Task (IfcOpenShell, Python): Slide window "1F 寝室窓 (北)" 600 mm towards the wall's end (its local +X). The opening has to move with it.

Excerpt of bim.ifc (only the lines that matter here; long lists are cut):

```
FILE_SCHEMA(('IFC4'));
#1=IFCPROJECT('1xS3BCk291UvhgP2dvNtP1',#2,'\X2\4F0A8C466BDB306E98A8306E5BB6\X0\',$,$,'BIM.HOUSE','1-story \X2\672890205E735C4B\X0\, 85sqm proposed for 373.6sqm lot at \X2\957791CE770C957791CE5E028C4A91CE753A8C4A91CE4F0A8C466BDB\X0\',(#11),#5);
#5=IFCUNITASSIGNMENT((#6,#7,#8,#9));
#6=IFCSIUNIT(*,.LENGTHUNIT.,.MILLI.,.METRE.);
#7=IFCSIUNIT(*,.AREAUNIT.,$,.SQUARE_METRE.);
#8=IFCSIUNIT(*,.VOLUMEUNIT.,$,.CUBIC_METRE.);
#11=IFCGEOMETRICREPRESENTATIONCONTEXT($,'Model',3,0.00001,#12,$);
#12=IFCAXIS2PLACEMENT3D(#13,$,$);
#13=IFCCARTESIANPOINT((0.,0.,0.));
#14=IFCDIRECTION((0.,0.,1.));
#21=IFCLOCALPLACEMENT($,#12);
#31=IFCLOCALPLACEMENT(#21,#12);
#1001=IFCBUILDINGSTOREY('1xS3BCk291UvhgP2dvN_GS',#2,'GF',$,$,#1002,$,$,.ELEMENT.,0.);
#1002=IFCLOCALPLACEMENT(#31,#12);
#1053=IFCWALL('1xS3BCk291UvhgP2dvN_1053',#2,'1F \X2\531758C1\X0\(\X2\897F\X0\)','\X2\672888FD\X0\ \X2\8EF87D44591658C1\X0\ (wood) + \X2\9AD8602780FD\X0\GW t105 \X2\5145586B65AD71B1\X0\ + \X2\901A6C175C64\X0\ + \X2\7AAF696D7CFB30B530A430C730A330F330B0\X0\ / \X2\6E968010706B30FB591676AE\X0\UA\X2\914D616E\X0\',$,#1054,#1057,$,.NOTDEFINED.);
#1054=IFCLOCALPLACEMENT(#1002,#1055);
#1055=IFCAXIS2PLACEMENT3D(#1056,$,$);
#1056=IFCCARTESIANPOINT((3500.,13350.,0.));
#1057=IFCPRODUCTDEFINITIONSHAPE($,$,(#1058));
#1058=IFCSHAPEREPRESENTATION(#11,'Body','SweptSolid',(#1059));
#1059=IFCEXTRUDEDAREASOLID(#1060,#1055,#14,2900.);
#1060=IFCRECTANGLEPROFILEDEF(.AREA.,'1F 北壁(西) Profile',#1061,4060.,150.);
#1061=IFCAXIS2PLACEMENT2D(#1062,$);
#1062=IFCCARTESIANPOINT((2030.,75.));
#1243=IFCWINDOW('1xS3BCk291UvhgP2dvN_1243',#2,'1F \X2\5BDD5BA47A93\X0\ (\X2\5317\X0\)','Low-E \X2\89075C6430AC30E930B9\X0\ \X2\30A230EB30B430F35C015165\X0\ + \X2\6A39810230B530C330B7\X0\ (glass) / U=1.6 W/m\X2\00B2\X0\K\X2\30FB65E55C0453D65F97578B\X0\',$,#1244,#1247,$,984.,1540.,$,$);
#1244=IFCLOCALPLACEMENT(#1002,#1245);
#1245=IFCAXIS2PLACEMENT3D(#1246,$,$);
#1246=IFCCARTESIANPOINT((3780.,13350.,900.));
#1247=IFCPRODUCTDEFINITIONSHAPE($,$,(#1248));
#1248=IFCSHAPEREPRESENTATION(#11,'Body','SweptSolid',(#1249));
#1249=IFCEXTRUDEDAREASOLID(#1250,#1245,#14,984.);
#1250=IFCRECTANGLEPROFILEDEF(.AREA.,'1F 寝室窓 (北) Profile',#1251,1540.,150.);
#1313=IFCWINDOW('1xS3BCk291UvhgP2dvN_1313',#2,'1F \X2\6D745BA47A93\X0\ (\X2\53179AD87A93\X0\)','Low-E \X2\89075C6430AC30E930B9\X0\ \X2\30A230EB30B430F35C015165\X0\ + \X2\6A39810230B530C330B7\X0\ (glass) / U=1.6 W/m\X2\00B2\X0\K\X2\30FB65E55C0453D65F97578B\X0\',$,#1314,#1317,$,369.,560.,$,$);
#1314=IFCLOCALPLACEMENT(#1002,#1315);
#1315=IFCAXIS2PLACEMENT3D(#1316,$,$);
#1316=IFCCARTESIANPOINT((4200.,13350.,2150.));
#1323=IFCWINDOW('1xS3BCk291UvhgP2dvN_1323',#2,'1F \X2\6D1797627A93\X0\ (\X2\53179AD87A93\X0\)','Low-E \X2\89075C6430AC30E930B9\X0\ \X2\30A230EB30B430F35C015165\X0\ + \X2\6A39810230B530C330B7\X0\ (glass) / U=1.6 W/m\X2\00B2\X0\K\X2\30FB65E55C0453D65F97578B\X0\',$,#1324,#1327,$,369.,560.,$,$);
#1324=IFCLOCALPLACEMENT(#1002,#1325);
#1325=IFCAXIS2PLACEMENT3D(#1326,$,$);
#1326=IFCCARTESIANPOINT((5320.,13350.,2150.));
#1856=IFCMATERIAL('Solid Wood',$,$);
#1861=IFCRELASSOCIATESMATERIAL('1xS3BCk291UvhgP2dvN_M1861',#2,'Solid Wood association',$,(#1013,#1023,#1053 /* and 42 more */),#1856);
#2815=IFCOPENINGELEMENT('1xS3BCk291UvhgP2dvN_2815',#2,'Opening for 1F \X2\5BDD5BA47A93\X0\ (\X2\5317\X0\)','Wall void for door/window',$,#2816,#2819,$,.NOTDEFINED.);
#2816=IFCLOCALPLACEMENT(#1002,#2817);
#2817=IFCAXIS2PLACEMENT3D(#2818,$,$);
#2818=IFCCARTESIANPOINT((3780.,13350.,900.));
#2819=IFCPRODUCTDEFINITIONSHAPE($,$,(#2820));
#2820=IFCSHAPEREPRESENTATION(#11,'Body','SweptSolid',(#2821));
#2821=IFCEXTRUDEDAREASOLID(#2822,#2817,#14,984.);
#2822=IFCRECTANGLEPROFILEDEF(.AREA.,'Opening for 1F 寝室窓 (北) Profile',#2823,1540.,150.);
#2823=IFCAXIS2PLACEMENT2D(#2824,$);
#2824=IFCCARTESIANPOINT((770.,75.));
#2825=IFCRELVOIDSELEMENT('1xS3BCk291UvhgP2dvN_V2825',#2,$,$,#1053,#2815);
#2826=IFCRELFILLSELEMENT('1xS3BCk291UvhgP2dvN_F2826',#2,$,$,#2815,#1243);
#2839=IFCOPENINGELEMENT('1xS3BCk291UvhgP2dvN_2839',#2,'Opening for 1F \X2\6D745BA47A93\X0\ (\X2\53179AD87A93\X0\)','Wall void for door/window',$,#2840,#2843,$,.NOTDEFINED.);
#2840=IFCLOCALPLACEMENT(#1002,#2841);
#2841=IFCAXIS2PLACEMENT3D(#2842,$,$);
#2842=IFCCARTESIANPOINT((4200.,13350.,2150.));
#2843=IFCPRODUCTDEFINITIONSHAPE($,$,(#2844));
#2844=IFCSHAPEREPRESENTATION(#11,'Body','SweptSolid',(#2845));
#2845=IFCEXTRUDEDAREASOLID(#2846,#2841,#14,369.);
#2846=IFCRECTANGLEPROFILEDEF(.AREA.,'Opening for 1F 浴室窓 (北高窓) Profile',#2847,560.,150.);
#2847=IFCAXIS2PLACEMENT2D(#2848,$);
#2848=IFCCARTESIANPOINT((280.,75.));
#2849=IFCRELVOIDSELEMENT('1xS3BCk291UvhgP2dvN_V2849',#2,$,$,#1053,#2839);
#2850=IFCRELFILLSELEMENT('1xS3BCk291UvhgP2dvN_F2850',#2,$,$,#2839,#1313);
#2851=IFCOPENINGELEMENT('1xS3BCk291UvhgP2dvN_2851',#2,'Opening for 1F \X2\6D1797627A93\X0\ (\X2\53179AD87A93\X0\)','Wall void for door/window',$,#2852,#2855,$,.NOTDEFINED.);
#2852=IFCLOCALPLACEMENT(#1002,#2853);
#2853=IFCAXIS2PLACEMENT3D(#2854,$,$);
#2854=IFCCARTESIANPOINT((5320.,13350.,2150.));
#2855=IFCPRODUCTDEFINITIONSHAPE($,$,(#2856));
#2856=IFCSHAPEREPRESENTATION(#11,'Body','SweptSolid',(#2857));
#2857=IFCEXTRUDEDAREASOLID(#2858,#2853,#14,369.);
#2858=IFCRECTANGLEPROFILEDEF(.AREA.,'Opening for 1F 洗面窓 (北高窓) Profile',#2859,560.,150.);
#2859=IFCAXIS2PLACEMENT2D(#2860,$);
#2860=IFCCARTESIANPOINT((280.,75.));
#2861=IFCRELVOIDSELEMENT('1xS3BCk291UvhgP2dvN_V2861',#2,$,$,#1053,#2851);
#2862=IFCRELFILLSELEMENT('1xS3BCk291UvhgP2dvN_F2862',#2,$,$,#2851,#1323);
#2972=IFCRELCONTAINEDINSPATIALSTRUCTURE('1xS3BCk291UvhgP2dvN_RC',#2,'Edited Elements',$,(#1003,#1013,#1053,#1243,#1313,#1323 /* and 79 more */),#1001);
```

```python
import ifcopenshell
import ifcopenshell.api.geometry
import ifcopenshell.util.placement
import ifcopenshell.util.unit

model = ifcopenshell.open("bim.ifc")
unit_scale = ifcopenshell.util.unit.calculate_unit_scale(model)

window = model.by_guid("1xS3BCk291UvhgP2dvN_1243")
opening = window.FillsVoids[0].RelatingOpeningElement
wall = opening.VoidsElements[0].RelatingBuildingElement

wall_matrix = ifcopenshell.util.placement.get_local_placement(wall.ObjectPlacement)
shift = wall_matrix[:3, 0] * 0.6 / unit_scale
before = ifcopenshell.util.placement.get_local_placement(window.ObjectPlacement)[:3, 3].copy()

# The window is not placed relative to its opening, so move both.
for product in (opening, window):
    matrix = ifcopenshell.util.placement.get_local_placement(product.ObjectPlacement)
    matrix[:3, 3] += shift
    ifcopenshell.api.geometry.edit_object_placement(model, product=product, matrix=matrix, is_si=False)

after = ifcopenshell.util.placement.get_local_placement(window.ObjectPlacement)[:3, 3]
print("window moved by", (after - before).round(3) + 0.0)

model.write("bim_updated.ifc")
```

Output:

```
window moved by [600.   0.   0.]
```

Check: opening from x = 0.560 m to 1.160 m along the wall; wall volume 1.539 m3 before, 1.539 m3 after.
